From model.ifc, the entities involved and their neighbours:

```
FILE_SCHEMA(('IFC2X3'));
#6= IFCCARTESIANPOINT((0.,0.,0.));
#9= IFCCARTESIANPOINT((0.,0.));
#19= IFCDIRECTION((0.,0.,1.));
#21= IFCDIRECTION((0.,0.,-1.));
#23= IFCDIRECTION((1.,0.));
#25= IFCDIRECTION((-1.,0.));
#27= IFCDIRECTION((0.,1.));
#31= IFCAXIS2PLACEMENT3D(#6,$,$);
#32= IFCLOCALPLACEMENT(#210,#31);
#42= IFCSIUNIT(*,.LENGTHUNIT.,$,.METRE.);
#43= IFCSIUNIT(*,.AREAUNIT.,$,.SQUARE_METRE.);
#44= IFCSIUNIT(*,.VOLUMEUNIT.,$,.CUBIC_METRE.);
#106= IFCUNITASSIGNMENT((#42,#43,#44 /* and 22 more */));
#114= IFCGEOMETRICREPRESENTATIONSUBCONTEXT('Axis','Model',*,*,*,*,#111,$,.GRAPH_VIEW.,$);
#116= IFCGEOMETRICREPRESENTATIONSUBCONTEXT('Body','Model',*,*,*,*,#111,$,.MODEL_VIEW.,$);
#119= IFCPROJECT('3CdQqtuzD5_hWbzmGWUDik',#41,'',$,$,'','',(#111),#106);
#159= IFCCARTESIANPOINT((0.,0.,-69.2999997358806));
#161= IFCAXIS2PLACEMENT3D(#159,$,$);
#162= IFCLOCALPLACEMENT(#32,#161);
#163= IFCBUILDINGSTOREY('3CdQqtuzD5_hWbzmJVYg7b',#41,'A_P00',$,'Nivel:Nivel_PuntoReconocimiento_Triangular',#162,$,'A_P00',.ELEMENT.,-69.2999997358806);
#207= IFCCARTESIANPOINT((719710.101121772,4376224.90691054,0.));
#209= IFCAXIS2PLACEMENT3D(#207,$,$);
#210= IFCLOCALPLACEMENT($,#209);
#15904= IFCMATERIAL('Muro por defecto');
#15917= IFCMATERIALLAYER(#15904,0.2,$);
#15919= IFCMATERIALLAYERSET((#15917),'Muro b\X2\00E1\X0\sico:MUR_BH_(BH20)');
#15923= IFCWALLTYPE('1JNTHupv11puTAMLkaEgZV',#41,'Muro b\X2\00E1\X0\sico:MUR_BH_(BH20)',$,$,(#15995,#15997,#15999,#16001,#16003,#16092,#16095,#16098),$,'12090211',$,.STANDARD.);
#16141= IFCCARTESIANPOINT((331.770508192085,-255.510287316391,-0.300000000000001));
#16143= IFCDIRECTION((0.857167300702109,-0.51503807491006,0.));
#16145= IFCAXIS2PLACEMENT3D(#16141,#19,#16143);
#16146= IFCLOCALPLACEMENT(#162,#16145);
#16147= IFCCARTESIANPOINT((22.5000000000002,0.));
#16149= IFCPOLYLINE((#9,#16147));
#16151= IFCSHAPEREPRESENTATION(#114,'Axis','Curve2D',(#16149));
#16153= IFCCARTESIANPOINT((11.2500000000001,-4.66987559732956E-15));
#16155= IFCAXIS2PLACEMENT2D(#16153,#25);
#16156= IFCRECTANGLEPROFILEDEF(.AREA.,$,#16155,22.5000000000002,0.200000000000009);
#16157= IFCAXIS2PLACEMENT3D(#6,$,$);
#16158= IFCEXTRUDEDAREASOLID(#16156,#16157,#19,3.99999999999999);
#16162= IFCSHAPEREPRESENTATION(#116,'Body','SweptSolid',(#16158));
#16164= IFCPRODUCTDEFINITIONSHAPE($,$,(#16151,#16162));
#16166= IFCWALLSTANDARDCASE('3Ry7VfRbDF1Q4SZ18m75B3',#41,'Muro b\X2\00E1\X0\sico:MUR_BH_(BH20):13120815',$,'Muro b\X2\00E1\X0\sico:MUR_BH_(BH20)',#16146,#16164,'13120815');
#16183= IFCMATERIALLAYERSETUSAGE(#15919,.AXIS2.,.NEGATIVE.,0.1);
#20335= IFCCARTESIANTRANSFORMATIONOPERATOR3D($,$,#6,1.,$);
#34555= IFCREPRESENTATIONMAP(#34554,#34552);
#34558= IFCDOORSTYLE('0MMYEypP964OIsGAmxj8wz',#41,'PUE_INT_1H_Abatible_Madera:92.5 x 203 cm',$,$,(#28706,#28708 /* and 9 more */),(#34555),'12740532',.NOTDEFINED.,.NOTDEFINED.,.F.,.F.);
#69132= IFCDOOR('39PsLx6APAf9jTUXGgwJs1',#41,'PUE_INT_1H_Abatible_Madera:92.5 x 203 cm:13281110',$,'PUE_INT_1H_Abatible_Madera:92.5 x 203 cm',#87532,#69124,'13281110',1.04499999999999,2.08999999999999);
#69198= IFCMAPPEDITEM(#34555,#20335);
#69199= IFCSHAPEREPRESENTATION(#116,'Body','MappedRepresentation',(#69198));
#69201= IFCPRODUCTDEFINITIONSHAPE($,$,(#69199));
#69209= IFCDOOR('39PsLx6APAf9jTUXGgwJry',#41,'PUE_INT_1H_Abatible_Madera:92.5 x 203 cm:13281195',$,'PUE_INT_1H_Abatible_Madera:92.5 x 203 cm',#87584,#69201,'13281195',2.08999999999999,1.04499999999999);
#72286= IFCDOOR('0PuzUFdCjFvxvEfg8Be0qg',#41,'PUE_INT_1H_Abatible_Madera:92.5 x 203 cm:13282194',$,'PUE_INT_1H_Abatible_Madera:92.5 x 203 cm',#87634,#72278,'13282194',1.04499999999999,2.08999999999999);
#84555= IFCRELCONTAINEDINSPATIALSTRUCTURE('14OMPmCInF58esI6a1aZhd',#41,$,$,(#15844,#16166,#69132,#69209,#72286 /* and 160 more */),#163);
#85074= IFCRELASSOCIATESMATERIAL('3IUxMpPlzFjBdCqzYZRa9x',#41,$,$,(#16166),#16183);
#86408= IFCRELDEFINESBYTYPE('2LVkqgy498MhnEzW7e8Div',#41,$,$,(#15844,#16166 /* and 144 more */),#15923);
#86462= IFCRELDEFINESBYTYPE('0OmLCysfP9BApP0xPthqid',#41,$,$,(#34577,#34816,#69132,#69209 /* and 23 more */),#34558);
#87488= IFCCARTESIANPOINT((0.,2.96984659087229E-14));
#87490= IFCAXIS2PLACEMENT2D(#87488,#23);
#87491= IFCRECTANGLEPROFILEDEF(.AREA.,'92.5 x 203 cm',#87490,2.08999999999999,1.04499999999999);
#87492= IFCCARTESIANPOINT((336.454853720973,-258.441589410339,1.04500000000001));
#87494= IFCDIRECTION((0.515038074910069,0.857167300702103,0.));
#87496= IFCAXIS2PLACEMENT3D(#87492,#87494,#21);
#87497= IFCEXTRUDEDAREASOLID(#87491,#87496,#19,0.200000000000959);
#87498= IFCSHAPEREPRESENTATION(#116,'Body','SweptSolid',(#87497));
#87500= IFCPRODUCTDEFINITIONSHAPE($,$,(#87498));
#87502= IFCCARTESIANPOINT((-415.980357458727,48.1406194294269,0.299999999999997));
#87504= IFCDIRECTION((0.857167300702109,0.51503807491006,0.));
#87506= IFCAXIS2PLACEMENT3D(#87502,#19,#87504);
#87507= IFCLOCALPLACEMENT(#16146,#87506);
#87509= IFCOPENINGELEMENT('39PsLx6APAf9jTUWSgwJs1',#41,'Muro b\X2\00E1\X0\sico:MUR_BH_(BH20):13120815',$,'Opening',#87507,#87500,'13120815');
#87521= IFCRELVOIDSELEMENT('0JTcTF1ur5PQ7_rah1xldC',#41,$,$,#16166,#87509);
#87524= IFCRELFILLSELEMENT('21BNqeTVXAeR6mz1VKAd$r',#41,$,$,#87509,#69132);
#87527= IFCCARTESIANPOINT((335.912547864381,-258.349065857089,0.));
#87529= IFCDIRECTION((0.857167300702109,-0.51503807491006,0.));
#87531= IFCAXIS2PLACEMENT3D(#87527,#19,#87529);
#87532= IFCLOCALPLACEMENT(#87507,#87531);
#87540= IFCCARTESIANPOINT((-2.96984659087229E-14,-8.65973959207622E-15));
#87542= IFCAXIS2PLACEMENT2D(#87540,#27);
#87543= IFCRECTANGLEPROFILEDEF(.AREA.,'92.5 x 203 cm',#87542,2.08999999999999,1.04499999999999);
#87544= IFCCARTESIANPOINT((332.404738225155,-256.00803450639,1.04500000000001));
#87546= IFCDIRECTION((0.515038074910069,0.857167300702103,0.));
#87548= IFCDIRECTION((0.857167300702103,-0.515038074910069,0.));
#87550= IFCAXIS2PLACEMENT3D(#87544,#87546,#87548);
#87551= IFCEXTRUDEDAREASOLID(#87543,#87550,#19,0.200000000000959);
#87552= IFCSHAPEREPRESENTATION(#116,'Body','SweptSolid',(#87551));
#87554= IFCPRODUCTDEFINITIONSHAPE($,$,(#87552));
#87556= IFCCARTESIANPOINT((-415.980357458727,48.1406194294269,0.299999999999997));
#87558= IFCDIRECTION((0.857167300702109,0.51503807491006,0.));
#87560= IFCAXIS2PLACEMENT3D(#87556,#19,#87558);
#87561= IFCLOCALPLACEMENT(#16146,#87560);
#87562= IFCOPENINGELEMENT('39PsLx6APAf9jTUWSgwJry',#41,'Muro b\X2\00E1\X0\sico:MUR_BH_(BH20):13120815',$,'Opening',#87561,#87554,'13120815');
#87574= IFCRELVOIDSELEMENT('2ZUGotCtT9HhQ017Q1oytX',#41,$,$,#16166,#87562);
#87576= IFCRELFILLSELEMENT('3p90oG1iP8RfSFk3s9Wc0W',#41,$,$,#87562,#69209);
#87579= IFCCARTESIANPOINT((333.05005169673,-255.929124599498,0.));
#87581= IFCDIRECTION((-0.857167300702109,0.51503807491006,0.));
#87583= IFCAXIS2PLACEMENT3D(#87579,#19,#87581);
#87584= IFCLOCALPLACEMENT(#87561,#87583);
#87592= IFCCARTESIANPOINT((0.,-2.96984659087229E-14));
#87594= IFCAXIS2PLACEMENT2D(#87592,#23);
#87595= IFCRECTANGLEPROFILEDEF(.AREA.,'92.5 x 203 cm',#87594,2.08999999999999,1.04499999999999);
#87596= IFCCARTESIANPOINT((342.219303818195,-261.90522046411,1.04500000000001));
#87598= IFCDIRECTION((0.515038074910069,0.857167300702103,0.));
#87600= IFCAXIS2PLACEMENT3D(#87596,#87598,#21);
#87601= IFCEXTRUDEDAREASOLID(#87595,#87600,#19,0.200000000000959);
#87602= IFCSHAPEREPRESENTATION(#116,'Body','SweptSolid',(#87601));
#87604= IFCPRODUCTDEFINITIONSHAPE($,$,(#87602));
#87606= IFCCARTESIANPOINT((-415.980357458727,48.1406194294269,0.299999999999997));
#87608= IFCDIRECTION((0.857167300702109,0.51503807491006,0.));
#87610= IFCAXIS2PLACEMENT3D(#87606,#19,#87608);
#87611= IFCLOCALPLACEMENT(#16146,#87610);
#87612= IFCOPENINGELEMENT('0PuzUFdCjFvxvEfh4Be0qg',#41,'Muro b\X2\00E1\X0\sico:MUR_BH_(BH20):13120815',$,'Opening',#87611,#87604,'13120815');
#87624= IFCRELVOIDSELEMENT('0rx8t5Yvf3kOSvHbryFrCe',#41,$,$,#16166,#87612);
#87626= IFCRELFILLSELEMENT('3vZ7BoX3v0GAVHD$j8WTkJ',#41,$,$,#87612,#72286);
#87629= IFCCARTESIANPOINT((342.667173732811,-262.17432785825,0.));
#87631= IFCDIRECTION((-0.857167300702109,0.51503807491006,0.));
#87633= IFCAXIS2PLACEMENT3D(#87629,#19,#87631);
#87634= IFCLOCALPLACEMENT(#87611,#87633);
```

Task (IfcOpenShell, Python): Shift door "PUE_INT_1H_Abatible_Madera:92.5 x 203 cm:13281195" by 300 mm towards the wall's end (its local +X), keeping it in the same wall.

```python
import ifcopenshell
import ifcopenshell.api.geometry
import ifcopenshell.util.placement
import ifcopenshell.util.unit

model = ifcopenshell.open("model.ifc")
unit_scale = ifcopenshell.util.unit.calculate_unit_scale(model)

door = model.by_guid("39PsLx6APAf9jTUXGgwJry")
opening = door.FillsVoids[0].RelatingOpeningElement
wall = opening.VoidsElements[0].RelatingBuildingElement

wall_matrix = ifcopenshell.util.placement.get_local_placement(wall.ObjectPlacement)
shift = wall_matrix[:3, 0] * 0.3 / unit_scale
before = ifcopenshell.util.placement.get_local_placement(door.ObjectPlacement)[:3, 3].copy()

# The door is placed relative to its opening, so it follows when the opening moves.
matrix = ifcopenshell.util.placement.get_local_placement(opening.ObjectPlacement)
matrix[:3, 3] += shift
ifcopenshell.api.geometry.edit_object_placement(
    model, product=opening, matrix=matrix, is_si=False, should_transform_children=True
)

after = ifcopenshell.util.placement.get_local_placement(door.ObjectPlacement)[:3, 3]
print("door moved by", (after - before).round(3) + 0.0)

model.write("model_edited.ifc")
```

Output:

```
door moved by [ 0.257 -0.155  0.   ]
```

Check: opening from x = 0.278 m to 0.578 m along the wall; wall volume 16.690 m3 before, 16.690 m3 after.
